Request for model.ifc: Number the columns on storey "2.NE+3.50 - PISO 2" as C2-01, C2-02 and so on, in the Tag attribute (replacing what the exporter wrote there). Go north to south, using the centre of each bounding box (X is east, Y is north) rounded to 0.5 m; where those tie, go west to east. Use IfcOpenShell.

First a look at what the model holds.

```python
import ifcopenshell
import ifcopenshell.util.element
import ifcopenshell.util.placement

model = ifcopenshell.open("model.ifc")
print(model.schema)
storey = next(s for s in model.by_type("IfcBuildingStorey") if s.Name == "2.NE+3.50 - PISO 2")
columns = [e for e in ifcopenshell.util.element.get_decomposition(storey) if e.is_a("IfcColumn")]
for e in sorted(columns, key=lambda e: e.id()):
    origin = ifcopenshell.util.placement.get_local_placement(e.ObjectPlacement)[:3, 3]
    print(e.id(), e.Tag, e.Name, origin.round(2) + 0.0, sep=" | ")
```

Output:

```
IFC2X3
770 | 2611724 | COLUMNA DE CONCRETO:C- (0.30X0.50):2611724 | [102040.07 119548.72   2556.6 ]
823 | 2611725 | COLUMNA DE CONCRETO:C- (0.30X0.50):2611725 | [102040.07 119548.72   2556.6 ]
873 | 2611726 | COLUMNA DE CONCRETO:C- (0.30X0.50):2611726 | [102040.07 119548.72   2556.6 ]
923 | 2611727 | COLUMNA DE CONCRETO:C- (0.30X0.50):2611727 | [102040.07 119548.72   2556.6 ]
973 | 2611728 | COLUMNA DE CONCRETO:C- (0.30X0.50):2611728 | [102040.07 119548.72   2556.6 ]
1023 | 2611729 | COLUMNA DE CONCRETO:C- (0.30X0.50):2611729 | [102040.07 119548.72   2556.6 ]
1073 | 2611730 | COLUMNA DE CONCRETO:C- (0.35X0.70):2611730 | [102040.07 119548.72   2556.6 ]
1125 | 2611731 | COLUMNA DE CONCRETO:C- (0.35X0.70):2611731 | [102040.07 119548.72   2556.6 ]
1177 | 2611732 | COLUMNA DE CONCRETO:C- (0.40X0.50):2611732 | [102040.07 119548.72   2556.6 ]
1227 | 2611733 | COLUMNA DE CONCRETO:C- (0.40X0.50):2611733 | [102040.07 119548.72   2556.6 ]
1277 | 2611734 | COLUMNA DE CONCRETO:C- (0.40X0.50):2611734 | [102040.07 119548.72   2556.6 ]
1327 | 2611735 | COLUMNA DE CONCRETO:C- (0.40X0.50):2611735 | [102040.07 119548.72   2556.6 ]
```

```python
import ifcopenshell
import ifcopenshell.geom
import ifcopenshell.util.element
import ifcopenshell.util.shape

model = ifcopenshell.open("model.ifc")
settings = ifcopenshell.geom.settings()
settings.set("use-world-coords", True)


def centre(element):
    shape = ifcopenshell.geom.create_shape(settings, element)
    return ifcopenshell.util.shape.get_bbox_centroid(shape.geometry)


storey = next(s for s in model.by_type("IfcBuildingStorey") if s.Name == "2.NE+3.50 - PISO 2")
columns = [e for e in ifcopenshell.util.element.get_decomposition(storey) if e.is_a("IfcColumn")]

# Insertion points can sit at a corner or the storey origin, so sort by the geometry (in metres).
centres = {e: centre(e) for e in columns}
columns.sort(key=lambda e: (-round(centres[e][1] / 0.5), centres[e][0]))

for i, e in enumerate(columns, start=1):
    number = f"C2-{i:02d}"
    e.Tag = number
    print(e.id(), number)

model.write("model_v2.ifc")
```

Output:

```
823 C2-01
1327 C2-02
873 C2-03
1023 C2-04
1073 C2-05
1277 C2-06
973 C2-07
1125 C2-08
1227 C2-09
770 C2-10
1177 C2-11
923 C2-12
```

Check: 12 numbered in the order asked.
